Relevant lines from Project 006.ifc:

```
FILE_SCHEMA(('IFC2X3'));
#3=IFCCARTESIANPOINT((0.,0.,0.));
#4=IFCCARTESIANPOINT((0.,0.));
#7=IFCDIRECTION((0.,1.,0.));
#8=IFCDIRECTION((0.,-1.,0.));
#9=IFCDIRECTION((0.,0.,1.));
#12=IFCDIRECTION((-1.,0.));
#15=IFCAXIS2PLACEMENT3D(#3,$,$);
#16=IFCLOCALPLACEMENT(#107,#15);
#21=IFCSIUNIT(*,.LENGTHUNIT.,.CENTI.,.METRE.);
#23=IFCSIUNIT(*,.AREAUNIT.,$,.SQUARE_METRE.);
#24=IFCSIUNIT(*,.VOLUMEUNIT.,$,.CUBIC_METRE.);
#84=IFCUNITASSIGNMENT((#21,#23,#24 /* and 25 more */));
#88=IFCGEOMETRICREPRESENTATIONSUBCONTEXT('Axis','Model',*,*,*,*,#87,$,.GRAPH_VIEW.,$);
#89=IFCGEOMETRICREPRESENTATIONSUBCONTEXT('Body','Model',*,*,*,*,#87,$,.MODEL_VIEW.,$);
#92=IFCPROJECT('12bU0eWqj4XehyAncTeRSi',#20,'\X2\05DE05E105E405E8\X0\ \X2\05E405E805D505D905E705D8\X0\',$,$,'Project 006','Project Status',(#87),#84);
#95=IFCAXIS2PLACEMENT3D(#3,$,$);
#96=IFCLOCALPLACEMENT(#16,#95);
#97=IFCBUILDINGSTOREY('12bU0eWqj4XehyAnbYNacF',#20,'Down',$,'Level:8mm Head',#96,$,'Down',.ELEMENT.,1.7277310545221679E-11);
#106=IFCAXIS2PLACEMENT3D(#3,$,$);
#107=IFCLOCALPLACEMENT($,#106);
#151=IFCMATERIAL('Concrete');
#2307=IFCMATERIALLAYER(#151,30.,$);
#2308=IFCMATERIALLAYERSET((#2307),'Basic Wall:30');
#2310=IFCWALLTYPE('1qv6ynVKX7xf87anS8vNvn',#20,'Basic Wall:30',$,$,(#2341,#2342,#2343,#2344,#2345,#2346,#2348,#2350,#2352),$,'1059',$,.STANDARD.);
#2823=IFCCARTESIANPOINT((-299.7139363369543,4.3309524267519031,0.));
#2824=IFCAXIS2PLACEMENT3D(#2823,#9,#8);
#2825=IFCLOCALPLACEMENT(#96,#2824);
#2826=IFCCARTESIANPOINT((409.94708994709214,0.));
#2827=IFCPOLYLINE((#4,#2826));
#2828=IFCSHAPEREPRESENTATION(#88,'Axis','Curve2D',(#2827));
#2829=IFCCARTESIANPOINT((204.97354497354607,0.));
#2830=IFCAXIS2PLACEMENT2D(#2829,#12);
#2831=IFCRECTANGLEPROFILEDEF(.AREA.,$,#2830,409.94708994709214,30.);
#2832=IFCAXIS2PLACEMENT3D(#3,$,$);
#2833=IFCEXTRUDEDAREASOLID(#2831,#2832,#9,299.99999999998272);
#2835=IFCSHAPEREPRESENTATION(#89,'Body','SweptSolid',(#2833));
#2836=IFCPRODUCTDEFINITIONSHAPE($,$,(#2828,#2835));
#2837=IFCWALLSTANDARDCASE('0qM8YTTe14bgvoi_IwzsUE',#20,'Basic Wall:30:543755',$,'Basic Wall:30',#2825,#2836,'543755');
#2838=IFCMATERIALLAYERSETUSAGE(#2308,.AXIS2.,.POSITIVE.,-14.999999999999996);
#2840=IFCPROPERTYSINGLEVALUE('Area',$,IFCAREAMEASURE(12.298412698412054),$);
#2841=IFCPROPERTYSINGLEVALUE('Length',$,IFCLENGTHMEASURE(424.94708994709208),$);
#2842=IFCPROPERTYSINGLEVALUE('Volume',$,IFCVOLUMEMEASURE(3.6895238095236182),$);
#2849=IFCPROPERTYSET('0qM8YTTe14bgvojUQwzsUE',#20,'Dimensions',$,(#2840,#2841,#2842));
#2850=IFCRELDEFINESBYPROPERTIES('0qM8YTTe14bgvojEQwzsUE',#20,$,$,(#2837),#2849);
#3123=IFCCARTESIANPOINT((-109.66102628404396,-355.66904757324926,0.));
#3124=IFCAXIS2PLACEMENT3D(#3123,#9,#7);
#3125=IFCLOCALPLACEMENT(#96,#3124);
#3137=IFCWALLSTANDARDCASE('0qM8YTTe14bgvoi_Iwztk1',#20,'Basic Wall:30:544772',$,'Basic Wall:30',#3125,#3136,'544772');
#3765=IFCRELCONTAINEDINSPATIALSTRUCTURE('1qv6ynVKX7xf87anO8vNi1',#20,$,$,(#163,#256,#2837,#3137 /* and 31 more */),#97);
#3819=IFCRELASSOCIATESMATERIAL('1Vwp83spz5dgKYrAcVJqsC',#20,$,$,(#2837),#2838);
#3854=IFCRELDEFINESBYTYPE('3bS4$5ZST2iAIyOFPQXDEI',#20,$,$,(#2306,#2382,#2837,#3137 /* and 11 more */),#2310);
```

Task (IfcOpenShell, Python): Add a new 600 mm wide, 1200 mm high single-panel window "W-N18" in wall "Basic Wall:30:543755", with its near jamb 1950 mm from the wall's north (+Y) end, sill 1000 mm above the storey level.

```python
import numpy as np
import ifcopenshell
import ifcopenshell.api.feature
import ifcopenshell.api.geometry
import ifcopenshell.api.pset
import ifcopenshell.api.root
import ifcopenshell.api.spatial
import ifcopenshell.api.type
import ifcopenshell.geom
import ifcopenshell.util.element
import ifcopenshell.util.placement
import ifcopenshell.util.representation
import ifcopenshell.util.shape
import ifcopenshell.util.unit

model = ifcopenshell.open("Project 006.ifc")
unit_scale = ifcopenshell.util.unit.calculate_unit_scale(model)
area_scale = ifcopenshell.util.unit.calculate_unit_scale(model, "AREAUNIT")
volume_scale = ifcopenshell.util.unit.calculate_unit_scale(model, "VOLUMEUNIT")
settings = ifcopenshell.geom.settings()


def volume(element):
    """Net volume in cubic metres, openings subtracted."""
    shape = ifcopenshell.geom.create_shape(settings, element)
    return ifcopenshell.util.shape.get_volume(shape.geometry)


wall = model.by_id(2837)
storey = ifcopenshell.util.element.get_container(wall, ifc_class="IfcBuildingStorey")
context = ifcopenshell.util.representation.get_context(model, "Model", "Body", "MODEL_VIEW")
before = volume(wall)

width, height, from_end, sill = 0.6, 1.2, 1.95, 1  # metres

# The wall runs along its own X axis, and the end named is its -X end.
wall_shape = ifcopenshell.geom.create_shape(settings, wall)
x, y, z = ifcopenshell.util.shape.get_vertices(wall_shape.geometry).T
start = x.min() + from_end
face, thickness = float(y.min()), float(y.max() - y.min())
wall_matrix = ifcopenshell.util.placement.get_local_placement(wall.ObjectPlacement)
level = ifcopenshell.util.placement.get_local_placement(storey.ObjectPlacement)[2, 3]


def in_wall(x, y):
    """Placement at x, y metres in the wall's axes, at sill height."""
    matrix = wall_matrix.copy()
    matrix[:, 3] = wall_matrix @ np.array([x / unit_scale, y / unit_scale, 0.0, 1.0])
    matrix[2, 3] = level + sill / unit_scale
    return matrix


# Opening: a box that overshoots both wall faces by 50 mm.
opening = ifcopenshell.api.root.create_entity(model, ifc_class="IfcOpeningElement")
box = ifcopenshell.api.geometry.add_wall_representation(
    model, context=context, length=width, height=height, thickness=thickness + 0.1
)
ifcopenshell.api.geometry.assign_representation(model, product=opening, representation=box)
ifcopenshell.api.geometry.edit_object_placement(model, product=opening, matrix=in_wall(start, face - 0.05), is_si=False)
ifcopenshell.api.feature.add_feature(model, feature=opening, element=wall)

window = ifcopenshell.api.root.create_entity(model, ifc_class="IfcWindow", name="W-N18")
window.OverallWidth, window.OverallHeight = width / unit_scale, height / unit_scale
body = ifcopenshell.api.geometry.add_window_representation(
    model,
    context=context,
    overall_width=window.OverallWidth,
    overall_height=window.OverallHeight,
    partition_type="SINGLE_PANEL",
)
ifcopenshell.api.geometry.assign_representation(model, product=window, representation=body)
ifcopenshell.api.spatial.assign_container(model, products=[window], relating_structure=storey)
fills = ifcopenshell.api.feature.add_filling(model, opening=opening, element=window)
fills.OwnerHistory = window.OwnerHistory  # required in IFC2X3

# IFC2X3 keeps the operation on the window style.
style = ifcopenshell.api.root.create_entity(model, ifc_class="IfcWindowStyle", name="W-N18")
style.OperationType, style.ConstructionType = "SINGLE_PANEL", "NOTDEFINED"
style.ParameterTakesPrecedence = style.Sizeable = False
ifcopenshell.api.type.assign_type(model, related_objects=[window], relating_type=style)

# Centre the window in the wall's thickness.
ifcopenshell.api.geometry.edit_object_placement(model, product=window, matrix=in_wall(start, face), is_si=False)
window_shape = ifcopenshell.geom.create_shape(settings, window)
depth = ifcopenshell.util.shape.get_vertices(window_shape.geometry)[:, 1]
offset = face + thickness / 2 - (depth.min() + depth.max()) / 2
ifcopenshell.api.geometry.edit_object_placement(model, product=window, matrix=in_wall(start, offset), is_si=False)

after = volume(wall)

# Update the wall's stored quantities.
pset = model.by_id(ifcopenshell.util.element.get_pset(wall, "Dimensions", should_inherit=False)["id"])
ifcopenshell.api.pset.edit_pset(model, pset=pset, properties={
    "Area": model.create_entity("IfcAreaMeasure", after / thickness / area_scale),
    "Volume": model.create_entity("IfcVolumeMeasure", after / volume_scale),
})

print(f"wall volume {before:.3f} -> {after:.3f} m3")

model.write("Project 006_rev.ifc")
```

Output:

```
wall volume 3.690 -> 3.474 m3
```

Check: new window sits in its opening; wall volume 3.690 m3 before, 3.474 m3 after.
